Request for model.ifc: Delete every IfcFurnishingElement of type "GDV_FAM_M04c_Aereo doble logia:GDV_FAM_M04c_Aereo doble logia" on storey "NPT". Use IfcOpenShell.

First a look at what the model holds.

```python
import ifcopenshell
import ifcopenshell.util.element

model = ifcopenshell.open("model.ifc")
print(model.schema)
storey = next(s for s in model.by_type("IfcBuildingStorey") if s.Name == "NPT")
furniture = [e for e in ifcopenshell.util.element.get_decomposition(storey) if e.is_a("IfcFurnishingElement")]
seen = {}
for e in furniture:
    element_type = ifcopenshell.util.element.get_type(e)
    name = element_type.Name if element_type not in (None, e) else None
    seen[name] = seen.get(name, 0) + 1
for name, count in sorted(seen.items(), key=str):
    print(count, "x", name)
```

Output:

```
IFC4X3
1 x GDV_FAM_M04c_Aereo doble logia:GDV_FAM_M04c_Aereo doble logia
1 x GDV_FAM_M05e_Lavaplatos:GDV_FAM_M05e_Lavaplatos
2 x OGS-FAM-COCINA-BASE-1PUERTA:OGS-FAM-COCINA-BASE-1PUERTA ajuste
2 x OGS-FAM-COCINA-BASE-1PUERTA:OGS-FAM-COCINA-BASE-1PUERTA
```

```python
import ifcopenshell
import ifcopenshell.api.root
import ifcopenshell.util.element

model = ifcopenshell.open("model.ifc")

storey = next(s for s in model.by_type("IfcBuildingStorey") if s.Name == "NPT")
furniture = [e for e in ifcopenshell.util.element.get_decomposition(storey) if e.is_a("IfcFurnishingElement")]
targets = [e for e in furniture if (t := ifcopenshell.util.element.get_type(e)) not in (None, e) and t.Name == "GDV_FAM_M04c_Aereo doble logia:GDV_FAM_M04c_Aereo doble logia"]

for e in targets:
    ifcopenshell.api.root.remove_product(model, product=e)
print(len(targets), "removed")

model.write("model_v2.ifc")
```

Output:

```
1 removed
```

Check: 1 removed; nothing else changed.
